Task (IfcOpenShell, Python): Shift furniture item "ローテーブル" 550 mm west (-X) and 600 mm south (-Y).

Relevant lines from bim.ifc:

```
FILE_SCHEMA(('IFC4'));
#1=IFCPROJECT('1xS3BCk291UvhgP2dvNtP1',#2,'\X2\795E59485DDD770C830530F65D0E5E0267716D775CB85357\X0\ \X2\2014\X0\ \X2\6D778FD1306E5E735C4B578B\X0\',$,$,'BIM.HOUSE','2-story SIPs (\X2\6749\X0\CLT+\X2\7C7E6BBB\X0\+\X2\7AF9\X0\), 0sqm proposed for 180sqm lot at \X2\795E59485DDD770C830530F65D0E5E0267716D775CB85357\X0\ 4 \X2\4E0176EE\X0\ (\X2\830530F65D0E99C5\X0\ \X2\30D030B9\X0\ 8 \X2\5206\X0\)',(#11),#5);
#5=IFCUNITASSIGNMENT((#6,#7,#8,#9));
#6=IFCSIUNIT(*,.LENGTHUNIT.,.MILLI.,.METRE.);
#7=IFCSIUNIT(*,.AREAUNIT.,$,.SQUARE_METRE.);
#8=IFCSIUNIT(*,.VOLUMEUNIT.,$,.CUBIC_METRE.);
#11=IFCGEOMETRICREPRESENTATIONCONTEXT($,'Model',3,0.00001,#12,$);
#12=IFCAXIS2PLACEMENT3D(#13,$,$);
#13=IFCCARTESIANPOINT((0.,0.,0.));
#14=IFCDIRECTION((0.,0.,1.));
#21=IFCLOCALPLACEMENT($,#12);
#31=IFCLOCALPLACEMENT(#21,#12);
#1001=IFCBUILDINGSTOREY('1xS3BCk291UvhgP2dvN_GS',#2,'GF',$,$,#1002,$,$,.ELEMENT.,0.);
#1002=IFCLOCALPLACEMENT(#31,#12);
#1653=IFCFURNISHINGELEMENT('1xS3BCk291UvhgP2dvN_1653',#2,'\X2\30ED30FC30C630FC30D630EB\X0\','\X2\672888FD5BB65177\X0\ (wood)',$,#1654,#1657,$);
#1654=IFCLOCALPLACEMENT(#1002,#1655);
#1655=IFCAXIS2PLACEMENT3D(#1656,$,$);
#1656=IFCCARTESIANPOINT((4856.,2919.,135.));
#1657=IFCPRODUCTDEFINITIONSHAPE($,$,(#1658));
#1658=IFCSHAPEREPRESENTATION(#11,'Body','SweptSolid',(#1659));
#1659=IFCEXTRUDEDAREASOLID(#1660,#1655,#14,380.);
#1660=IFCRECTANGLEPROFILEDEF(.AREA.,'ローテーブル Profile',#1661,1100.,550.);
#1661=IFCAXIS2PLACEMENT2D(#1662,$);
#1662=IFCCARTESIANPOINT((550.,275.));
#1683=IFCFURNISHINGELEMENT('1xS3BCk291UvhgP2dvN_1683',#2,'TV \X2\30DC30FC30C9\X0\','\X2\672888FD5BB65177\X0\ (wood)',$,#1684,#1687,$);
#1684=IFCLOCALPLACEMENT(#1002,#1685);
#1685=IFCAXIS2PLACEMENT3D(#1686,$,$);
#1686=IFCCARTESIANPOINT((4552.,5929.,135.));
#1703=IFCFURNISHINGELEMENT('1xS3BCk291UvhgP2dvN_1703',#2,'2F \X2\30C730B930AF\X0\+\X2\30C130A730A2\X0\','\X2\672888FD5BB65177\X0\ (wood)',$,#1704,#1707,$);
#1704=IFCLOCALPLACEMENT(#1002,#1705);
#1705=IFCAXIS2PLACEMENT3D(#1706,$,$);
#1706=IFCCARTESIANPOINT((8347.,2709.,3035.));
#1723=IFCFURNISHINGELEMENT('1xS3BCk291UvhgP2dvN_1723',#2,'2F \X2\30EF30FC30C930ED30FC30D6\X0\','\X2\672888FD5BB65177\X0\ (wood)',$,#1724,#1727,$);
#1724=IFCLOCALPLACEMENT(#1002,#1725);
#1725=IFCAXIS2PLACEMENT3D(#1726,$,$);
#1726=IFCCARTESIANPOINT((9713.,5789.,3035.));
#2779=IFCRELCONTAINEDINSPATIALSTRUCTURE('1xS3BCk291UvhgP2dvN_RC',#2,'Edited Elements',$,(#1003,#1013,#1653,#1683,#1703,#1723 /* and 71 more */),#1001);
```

```python
import ifcopenshell
import ifcopenshell.api.geometry
import ifcopenshell.util.placement

model = ifcopenshell.open("bim.ifc")

item = model.by_guid("1xS3BCk291UvhgP2dvN_1653")
matrix = ifcopenshell.util.placement.get_local_placement(item.ObjectPlacement)
matrix[0, 3] -= 550.0
matrix[1, 3] -= 600.0
ifcopenshell.api.geometry.edit_object_placement(model, product=item, matrix=matrix, is_si=False)

print(ifcopenshell.util.placement.get_local_placement(item.ObjectPlacement).round(3) + 0.0)

model.write("bim_updated.ifc")
```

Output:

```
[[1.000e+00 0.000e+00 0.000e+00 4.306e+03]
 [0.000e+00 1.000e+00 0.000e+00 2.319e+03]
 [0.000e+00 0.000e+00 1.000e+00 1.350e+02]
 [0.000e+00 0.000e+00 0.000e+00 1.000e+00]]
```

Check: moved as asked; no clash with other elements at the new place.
